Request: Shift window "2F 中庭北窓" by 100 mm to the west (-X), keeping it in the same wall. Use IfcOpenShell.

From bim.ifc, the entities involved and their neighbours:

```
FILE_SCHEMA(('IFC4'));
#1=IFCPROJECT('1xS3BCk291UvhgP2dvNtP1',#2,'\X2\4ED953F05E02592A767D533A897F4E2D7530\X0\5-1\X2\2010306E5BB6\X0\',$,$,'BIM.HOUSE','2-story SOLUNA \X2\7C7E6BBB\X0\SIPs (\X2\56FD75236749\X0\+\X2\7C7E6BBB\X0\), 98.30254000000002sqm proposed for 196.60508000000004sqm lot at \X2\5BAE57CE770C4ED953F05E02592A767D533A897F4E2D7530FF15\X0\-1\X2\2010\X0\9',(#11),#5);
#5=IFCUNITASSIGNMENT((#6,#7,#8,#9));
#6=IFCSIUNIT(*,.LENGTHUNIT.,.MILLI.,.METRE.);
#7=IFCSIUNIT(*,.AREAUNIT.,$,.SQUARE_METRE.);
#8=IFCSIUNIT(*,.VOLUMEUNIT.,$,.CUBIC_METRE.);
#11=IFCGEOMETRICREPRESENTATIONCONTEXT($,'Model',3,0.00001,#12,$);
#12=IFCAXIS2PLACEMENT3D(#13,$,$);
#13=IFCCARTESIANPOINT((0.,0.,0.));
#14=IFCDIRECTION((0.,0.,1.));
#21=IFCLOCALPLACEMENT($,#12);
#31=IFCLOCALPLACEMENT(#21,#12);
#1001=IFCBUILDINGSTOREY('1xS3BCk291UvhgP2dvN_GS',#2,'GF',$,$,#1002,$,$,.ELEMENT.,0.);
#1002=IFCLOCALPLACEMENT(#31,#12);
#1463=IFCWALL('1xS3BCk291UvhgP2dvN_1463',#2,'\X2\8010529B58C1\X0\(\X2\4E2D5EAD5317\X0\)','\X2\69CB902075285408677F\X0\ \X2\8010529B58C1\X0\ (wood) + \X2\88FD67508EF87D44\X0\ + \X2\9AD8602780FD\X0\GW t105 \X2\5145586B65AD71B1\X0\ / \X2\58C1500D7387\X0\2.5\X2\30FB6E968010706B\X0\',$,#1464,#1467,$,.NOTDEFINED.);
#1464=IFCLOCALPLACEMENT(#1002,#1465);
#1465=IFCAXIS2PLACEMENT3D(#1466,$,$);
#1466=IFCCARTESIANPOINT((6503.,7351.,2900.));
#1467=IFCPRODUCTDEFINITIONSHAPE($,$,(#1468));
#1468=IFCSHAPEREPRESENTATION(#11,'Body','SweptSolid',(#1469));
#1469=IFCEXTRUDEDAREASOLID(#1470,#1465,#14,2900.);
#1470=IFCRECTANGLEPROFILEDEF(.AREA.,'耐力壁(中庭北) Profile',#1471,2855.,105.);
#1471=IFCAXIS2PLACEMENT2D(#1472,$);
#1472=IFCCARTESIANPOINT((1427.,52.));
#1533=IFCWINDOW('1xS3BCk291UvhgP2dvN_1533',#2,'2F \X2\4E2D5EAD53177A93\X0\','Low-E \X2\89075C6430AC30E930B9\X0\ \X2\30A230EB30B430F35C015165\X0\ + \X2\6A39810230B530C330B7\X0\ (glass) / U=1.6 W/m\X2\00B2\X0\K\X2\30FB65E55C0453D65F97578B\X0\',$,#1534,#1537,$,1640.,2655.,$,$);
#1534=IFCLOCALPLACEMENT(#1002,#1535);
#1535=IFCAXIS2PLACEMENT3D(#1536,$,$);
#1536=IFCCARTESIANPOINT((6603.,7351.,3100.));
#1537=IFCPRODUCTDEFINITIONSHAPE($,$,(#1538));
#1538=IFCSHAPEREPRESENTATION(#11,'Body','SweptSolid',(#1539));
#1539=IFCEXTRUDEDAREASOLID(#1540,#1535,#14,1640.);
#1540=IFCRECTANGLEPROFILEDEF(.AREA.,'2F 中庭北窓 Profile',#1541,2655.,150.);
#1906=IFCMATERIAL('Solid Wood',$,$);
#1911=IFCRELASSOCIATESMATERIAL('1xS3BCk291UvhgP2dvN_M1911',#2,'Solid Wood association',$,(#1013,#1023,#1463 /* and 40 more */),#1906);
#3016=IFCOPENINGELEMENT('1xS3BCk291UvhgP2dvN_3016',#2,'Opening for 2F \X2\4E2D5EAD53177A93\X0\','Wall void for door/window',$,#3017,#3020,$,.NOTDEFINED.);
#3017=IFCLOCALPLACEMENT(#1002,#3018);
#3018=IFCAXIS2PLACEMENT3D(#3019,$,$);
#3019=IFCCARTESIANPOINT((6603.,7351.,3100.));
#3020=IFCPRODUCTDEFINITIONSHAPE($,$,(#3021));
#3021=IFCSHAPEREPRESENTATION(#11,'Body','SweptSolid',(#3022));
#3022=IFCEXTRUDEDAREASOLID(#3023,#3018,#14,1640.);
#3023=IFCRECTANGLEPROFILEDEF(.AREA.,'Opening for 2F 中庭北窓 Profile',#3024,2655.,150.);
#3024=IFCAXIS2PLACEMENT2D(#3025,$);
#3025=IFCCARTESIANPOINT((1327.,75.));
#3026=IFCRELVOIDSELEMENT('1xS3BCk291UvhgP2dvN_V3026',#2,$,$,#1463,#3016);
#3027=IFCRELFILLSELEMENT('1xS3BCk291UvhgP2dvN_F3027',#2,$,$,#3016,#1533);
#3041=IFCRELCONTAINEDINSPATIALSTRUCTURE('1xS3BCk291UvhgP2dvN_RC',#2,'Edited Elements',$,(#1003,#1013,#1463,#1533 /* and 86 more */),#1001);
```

```python
import ifcopenshell
import ifcopenshell.api.geometry
import ifcopenshell.util.placement
import ifcopenshell.util.unit

model = ifcopenshell.open("bim.ifc")
unit_scale = ifcopenshell.util.unit.calculate_unit_scale(model)

window = model.by_guid("1xS3BCk291UvhgP2dvN_1533")
opening = window.FillsVoids[0].RelatingOpeningElement
wall = opening.VoidsElements[0].RelatingBuildingElement

wall_matrix = ifcopenshell.util.placement.get_local_placement(wall.ObjectPlacement)
shift = wall_matrix[:3, 0] * -0.1 / unit_scale
before = ifcopenshell.util.placement.get_local_placement(window.ObjectPlacement)[:3, 3].copy()

# The window is not placed relative to its opening, so move both.
for product in (opening, window):
    matrix = ifcopenshell.util.placement.get_local_placement(product.ObjectPlacement)
    matrix[:3, 3] += shift
    ifcopenshell.api.geometry.edit_object_placement(model, product=product, matrix=matrix, is_si=False)

after = ifcopenshell.util.placement.get_local_placement(window.ObjectPlacement)[:3, 3]
print("window moved by", (after - before).round(3) + 0.0)

model.write("bim_updated.ifc")
```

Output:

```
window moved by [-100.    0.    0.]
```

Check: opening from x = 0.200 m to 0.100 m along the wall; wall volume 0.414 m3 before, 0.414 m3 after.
